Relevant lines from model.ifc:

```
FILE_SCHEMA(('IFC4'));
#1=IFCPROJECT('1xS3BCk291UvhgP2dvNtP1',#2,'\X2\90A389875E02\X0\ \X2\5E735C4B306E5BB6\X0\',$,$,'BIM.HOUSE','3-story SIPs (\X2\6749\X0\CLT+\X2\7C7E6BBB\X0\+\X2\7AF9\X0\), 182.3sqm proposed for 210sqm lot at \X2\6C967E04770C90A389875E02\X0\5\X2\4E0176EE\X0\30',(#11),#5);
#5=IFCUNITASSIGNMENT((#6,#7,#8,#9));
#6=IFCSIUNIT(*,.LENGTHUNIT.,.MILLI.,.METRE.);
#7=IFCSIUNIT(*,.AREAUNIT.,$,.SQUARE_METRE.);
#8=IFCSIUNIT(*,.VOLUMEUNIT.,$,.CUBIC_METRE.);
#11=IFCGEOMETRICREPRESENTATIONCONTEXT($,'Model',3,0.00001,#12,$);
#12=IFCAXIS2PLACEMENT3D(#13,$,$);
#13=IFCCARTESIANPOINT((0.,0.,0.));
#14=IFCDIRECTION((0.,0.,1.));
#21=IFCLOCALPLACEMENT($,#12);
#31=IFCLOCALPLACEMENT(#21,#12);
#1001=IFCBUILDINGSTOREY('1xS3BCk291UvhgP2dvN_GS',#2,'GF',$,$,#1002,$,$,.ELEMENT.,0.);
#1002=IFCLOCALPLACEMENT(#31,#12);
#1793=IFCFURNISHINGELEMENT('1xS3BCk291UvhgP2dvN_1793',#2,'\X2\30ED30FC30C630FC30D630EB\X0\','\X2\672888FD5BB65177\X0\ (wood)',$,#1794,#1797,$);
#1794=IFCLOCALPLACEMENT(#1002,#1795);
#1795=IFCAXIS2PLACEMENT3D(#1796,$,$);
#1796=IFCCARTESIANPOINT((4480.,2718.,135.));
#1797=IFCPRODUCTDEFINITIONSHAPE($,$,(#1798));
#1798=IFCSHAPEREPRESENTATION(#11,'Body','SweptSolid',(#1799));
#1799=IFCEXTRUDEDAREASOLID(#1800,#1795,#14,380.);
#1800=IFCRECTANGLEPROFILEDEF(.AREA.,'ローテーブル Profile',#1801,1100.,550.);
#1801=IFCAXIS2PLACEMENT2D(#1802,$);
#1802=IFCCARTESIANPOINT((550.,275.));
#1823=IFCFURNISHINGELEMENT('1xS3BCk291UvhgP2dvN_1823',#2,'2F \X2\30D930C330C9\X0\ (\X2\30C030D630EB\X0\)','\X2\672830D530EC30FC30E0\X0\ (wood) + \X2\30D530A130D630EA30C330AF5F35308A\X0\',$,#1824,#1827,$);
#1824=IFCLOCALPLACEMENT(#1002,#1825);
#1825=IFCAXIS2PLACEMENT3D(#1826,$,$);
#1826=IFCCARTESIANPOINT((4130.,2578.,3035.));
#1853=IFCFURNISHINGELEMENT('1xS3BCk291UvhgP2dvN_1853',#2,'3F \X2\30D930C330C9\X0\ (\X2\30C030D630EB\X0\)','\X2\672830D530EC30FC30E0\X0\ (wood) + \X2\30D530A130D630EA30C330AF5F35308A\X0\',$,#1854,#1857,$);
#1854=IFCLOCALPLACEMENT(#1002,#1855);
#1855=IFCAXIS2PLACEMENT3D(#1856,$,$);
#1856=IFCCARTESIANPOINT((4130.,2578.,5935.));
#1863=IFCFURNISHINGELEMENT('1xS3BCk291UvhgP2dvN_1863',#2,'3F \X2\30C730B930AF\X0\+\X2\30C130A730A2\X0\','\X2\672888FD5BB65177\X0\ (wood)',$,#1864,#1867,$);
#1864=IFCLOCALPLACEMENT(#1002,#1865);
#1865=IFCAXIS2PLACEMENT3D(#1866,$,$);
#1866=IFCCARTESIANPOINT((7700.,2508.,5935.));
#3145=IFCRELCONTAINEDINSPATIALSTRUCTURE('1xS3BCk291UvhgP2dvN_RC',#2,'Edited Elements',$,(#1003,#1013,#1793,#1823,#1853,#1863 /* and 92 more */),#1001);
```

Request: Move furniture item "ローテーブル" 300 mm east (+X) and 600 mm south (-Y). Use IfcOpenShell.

```python
import ifcopenshell
import ifcopenshell.api.geometry
import ifcopenshell.util.placement
import ifcopenshell.util.unit

model = ifcopenshell.open("model.ifc")
unit_scale = ifcopenshell.util.unit.calculate_unit_scale(model)

item = model.by_guid("1xS3BCk291UvhgP2dvN_1793")
matrix = ifcopenshell.util.placement.get_local_placement(item.ObjectPlacement)
matrix[0, 3] += 0.3 / unit_scale
matrix[1, 3] -= 0.6 / unit_scale
ifcopenshell.api.geometry.edit_object_placement(model, product=item, matrix=matrix, is_si=False)

print(ifcopenshell.util.placement.get_local_placement(item.ObjectPlacement).round(3) + 0.0)

model.write("model_updated.ifc")
```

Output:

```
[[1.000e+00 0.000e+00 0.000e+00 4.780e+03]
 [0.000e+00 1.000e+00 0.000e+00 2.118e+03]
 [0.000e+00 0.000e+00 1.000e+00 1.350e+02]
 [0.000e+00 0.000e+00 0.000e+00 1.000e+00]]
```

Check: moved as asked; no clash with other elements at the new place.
